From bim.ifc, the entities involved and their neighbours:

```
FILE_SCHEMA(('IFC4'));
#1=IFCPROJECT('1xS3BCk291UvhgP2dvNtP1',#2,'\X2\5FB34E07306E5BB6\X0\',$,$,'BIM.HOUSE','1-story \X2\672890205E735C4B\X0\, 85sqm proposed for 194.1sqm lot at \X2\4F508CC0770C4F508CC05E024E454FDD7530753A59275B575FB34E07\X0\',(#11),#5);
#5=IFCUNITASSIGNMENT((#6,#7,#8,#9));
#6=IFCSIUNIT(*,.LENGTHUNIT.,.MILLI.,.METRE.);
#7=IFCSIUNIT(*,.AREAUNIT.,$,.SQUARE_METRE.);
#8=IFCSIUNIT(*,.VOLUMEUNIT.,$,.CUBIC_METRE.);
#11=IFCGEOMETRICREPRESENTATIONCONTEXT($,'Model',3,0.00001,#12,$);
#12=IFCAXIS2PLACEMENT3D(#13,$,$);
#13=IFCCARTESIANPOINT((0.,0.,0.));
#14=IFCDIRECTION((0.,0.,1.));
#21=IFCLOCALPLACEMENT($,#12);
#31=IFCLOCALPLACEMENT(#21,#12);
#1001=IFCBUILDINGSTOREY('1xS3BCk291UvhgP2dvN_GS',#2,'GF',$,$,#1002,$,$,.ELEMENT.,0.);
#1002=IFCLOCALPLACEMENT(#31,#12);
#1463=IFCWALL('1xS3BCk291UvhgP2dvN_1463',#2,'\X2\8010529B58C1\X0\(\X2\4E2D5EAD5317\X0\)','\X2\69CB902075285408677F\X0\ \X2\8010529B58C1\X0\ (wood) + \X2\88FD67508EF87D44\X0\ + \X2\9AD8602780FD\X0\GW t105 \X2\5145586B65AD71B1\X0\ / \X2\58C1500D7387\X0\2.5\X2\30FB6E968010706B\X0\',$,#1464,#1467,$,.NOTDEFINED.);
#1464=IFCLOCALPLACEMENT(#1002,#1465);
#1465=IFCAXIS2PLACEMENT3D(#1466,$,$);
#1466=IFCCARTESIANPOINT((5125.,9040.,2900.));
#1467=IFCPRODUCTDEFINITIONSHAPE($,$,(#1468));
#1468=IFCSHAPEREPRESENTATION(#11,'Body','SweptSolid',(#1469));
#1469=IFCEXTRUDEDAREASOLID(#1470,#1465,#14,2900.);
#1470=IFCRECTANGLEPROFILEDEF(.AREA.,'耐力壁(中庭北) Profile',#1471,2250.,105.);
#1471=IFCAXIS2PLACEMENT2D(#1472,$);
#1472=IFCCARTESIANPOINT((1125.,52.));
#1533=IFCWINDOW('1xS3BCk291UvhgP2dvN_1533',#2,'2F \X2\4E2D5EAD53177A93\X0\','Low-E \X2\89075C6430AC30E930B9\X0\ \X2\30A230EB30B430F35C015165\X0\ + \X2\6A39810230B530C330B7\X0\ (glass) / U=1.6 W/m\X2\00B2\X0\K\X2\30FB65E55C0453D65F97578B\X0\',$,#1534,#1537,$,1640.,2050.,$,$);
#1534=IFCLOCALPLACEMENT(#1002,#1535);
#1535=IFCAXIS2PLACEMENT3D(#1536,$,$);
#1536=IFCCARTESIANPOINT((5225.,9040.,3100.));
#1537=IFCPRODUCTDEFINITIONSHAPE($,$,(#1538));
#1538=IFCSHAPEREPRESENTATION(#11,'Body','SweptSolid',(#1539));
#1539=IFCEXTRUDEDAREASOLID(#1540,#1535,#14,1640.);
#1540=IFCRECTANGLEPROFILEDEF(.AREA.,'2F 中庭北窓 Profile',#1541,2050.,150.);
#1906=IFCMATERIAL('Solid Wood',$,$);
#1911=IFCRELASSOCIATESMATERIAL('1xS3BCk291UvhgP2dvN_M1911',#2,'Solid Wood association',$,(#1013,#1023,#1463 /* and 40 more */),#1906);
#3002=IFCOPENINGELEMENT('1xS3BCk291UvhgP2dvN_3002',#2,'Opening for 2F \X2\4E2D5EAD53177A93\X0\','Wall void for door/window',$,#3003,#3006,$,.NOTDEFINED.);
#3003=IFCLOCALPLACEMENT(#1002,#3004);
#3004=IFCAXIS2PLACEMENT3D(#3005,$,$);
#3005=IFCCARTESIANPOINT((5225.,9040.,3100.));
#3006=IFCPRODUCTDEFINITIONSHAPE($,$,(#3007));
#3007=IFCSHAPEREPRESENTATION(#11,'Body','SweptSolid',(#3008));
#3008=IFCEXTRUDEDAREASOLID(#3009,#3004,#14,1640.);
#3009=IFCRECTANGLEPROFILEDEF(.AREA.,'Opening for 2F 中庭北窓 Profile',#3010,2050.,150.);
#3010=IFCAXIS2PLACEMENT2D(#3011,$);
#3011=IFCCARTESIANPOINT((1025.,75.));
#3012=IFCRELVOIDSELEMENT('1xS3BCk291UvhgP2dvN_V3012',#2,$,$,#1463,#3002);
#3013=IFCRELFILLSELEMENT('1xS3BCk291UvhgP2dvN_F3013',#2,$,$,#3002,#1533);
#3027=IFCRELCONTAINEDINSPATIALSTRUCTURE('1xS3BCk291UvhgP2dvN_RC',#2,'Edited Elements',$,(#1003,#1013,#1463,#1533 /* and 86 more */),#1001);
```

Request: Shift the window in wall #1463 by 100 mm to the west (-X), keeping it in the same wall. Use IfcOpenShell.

```python
import ifcopenshell
import ifcopenshell.api.geometry
import ifcopenshell.util.placement
import ifcopenshell.util.unit

model = ifcopenshell.open("bim.ifc")
unit_scale = ifcopenshell.util.unit.calculate_unit_scale(model)

window = model.by_id(1533)
opening = window.FillsVoids[0].RelatingOpeningElement
wall = opening.VoidsElements[0].RelatingBuildingElement

wall_matrix = ifcopenshell.util.placement.get_local_placement(wall.ObjectPlacement)
shift = wall_matrix[:3, 0] * -0.1 / unit_scale
before = ifcopenshell.util.placement.get_local_placement(window.ObjectPlacement)[:3, 3].copy()

# The window is not placed relative to its opening, so move both.
for product in (opening, window):
    matrix = ifcopenshell.util.placement.get_local_placement(product.ObjectPlacement)
    matrix[:3, 3] += shift
    ifcopenshell.api.geometry.edit_object_placement(model, product=product, matrix=matrix, is_si=False)

after = ifcopenshell.util.placement.get_local_placement(window.ObjectPlacement)[:3, 3]
print("window moved by", (after - before).round(3) + 0.0)

model.write("bim_v2.ifc")
```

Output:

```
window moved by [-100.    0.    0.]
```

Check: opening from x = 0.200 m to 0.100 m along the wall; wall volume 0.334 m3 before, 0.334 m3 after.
